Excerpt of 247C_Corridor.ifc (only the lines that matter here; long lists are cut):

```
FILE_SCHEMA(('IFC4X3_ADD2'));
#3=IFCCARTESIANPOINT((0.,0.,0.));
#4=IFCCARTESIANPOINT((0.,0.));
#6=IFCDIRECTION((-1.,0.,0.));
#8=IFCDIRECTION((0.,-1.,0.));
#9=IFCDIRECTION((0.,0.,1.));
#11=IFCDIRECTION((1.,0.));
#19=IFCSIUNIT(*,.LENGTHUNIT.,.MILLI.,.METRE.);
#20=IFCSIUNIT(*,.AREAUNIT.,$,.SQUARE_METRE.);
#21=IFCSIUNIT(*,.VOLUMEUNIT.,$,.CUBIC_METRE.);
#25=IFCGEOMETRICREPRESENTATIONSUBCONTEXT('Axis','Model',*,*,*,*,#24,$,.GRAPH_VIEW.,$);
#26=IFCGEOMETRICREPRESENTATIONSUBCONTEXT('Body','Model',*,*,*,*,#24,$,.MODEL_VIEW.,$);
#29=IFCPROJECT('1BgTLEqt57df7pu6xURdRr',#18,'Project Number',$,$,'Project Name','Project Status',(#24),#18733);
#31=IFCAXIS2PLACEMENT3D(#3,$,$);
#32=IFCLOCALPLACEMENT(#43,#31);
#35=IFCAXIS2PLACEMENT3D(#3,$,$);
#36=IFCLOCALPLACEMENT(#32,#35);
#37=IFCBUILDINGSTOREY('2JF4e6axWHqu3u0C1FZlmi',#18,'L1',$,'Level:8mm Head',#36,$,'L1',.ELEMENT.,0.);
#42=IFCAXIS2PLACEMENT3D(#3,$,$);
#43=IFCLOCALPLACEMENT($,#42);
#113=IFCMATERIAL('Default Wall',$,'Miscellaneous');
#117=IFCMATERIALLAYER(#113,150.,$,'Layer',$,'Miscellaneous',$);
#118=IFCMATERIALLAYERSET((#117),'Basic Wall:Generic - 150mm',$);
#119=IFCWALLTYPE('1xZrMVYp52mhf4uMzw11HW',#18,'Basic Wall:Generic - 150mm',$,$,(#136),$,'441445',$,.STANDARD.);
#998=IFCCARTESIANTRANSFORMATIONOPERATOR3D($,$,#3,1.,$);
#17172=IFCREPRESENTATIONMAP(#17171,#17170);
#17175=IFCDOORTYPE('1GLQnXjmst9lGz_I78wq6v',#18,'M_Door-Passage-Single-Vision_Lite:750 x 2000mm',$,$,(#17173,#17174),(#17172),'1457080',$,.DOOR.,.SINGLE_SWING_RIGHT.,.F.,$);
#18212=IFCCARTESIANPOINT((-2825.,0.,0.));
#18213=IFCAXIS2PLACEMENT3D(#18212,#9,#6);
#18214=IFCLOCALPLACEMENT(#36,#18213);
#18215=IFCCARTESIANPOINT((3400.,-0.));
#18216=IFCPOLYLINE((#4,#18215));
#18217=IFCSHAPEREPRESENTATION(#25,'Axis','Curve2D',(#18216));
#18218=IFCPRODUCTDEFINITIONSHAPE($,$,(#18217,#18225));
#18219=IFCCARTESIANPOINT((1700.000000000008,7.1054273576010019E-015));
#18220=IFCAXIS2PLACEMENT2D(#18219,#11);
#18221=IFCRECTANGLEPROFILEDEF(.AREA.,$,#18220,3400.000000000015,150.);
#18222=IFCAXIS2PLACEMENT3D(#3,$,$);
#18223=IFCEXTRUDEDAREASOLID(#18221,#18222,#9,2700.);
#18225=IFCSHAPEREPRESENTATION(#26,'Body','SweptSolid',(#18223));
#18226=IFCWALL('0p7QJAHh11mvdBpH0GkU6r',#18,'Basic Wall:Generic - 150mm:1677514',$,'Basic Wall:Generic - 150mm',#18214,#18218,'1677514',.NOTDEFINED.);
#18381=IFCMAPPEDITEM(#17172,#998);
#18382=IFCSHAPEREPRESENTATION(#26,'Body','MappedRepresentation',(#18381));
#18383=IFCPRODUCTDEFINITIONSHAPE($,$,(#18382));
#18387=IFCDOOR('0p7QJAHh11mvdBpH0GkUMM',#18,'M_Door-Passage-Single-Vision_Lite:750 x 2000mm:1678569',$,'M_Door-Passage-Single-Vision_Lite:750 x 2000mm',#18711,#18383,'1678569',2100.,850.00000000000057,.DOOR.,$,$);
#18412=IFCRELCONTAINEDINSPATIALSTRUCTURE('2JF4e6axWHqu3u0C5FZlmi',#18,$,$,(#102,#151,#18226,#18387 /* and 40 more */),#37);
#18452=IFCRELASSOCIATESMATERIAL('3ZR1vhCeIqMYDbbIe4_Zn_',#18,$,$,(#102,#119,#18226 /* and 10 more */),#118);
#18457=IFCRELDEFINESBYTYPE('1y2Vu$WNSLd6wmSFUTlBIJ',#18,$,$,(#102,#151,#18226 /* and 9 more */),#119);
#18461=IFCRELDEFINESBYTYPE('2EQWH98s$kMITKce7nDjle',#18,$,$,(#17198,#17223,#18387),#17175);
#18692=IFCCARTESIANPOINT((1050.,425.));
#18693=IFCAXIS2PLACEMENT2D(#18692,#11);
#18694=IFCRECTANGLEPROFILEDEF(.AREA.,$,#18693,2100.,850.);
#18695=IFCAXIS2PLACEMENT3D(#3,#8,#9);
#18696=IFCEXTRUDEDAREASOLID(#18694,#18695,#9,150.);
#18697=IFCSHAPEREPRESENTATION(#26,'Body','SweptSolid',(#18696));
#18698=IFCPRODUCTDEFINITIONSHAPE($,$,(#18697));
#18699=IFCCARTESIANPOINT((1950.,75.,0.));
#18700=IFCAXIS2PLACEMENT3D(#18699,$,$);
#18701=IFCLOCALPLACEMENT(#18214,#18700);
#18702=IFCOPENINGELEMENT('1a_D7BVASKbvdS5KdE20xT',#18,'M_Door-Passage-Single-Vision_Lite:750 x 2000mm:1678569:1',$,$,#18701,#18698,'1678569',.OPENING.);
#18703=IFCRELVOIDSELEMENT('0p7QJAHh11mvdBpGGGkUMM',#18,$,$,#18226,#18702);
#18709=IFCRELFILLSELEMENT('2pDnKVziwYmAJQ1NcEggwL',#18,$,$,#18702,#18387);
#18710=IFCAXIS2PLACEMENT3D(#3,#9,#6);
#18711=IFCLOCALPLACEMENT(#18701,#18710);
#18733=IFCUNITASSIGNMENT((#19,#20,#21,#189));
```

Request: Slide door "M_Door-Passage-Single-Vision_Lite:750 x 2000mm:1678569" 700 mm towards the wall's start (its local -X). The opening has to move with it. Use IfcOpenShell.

```python
import ifcopenshell
import ifcopenshell.api.geometry
import ifcopenshell.util.placement
import ifcopenshell.util.unit

model = ifcopenshell.open("247C_Corridor.ifc")
unit_scale = ifcopenshell.util.unit.calculate_unit_scale(model)

door = model.by_guid("0p7QJAHh11mvdBpH0GkUMM")
opening = door.FillsVoids[0].RelatingOpeningElement
wall = opening.VoidsElements[0].RelatingBuildingElement

wall_matrix = ifcopenshell.util.placement.get_local_placement(wall.ObjectPlacement)
shift = wall_matrix[:3, 0] * -0.7 / unit_scale
before = ifcopenshell.util.placement.get_local_placement(door.ObjectPlacement)[:3, 3].copy()

# The door is placed relative to its opening, so it follows when the opening moves.
matrix = ifcopenshell.util.placement.get_local_placement(opening.ObjectPlacement)
matrix[:3, 3] += shift
ifcopenshell.api.geometry.edit_object_placement(
    model, product=opening, matrix=matrix, is_si=False, should_transform_children=True
)

after = ifcopenshell.util.placement.get_local_placement(door.ObjectPlacement)[:3, 3]
print("door moved by", (after - before).round(3) + 0.0)

model.write("247C_Corridor_rev.ifc")
```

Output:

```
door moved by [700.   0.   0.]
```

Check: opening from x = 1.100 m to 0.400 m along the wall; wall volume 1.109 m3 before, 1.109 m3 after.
